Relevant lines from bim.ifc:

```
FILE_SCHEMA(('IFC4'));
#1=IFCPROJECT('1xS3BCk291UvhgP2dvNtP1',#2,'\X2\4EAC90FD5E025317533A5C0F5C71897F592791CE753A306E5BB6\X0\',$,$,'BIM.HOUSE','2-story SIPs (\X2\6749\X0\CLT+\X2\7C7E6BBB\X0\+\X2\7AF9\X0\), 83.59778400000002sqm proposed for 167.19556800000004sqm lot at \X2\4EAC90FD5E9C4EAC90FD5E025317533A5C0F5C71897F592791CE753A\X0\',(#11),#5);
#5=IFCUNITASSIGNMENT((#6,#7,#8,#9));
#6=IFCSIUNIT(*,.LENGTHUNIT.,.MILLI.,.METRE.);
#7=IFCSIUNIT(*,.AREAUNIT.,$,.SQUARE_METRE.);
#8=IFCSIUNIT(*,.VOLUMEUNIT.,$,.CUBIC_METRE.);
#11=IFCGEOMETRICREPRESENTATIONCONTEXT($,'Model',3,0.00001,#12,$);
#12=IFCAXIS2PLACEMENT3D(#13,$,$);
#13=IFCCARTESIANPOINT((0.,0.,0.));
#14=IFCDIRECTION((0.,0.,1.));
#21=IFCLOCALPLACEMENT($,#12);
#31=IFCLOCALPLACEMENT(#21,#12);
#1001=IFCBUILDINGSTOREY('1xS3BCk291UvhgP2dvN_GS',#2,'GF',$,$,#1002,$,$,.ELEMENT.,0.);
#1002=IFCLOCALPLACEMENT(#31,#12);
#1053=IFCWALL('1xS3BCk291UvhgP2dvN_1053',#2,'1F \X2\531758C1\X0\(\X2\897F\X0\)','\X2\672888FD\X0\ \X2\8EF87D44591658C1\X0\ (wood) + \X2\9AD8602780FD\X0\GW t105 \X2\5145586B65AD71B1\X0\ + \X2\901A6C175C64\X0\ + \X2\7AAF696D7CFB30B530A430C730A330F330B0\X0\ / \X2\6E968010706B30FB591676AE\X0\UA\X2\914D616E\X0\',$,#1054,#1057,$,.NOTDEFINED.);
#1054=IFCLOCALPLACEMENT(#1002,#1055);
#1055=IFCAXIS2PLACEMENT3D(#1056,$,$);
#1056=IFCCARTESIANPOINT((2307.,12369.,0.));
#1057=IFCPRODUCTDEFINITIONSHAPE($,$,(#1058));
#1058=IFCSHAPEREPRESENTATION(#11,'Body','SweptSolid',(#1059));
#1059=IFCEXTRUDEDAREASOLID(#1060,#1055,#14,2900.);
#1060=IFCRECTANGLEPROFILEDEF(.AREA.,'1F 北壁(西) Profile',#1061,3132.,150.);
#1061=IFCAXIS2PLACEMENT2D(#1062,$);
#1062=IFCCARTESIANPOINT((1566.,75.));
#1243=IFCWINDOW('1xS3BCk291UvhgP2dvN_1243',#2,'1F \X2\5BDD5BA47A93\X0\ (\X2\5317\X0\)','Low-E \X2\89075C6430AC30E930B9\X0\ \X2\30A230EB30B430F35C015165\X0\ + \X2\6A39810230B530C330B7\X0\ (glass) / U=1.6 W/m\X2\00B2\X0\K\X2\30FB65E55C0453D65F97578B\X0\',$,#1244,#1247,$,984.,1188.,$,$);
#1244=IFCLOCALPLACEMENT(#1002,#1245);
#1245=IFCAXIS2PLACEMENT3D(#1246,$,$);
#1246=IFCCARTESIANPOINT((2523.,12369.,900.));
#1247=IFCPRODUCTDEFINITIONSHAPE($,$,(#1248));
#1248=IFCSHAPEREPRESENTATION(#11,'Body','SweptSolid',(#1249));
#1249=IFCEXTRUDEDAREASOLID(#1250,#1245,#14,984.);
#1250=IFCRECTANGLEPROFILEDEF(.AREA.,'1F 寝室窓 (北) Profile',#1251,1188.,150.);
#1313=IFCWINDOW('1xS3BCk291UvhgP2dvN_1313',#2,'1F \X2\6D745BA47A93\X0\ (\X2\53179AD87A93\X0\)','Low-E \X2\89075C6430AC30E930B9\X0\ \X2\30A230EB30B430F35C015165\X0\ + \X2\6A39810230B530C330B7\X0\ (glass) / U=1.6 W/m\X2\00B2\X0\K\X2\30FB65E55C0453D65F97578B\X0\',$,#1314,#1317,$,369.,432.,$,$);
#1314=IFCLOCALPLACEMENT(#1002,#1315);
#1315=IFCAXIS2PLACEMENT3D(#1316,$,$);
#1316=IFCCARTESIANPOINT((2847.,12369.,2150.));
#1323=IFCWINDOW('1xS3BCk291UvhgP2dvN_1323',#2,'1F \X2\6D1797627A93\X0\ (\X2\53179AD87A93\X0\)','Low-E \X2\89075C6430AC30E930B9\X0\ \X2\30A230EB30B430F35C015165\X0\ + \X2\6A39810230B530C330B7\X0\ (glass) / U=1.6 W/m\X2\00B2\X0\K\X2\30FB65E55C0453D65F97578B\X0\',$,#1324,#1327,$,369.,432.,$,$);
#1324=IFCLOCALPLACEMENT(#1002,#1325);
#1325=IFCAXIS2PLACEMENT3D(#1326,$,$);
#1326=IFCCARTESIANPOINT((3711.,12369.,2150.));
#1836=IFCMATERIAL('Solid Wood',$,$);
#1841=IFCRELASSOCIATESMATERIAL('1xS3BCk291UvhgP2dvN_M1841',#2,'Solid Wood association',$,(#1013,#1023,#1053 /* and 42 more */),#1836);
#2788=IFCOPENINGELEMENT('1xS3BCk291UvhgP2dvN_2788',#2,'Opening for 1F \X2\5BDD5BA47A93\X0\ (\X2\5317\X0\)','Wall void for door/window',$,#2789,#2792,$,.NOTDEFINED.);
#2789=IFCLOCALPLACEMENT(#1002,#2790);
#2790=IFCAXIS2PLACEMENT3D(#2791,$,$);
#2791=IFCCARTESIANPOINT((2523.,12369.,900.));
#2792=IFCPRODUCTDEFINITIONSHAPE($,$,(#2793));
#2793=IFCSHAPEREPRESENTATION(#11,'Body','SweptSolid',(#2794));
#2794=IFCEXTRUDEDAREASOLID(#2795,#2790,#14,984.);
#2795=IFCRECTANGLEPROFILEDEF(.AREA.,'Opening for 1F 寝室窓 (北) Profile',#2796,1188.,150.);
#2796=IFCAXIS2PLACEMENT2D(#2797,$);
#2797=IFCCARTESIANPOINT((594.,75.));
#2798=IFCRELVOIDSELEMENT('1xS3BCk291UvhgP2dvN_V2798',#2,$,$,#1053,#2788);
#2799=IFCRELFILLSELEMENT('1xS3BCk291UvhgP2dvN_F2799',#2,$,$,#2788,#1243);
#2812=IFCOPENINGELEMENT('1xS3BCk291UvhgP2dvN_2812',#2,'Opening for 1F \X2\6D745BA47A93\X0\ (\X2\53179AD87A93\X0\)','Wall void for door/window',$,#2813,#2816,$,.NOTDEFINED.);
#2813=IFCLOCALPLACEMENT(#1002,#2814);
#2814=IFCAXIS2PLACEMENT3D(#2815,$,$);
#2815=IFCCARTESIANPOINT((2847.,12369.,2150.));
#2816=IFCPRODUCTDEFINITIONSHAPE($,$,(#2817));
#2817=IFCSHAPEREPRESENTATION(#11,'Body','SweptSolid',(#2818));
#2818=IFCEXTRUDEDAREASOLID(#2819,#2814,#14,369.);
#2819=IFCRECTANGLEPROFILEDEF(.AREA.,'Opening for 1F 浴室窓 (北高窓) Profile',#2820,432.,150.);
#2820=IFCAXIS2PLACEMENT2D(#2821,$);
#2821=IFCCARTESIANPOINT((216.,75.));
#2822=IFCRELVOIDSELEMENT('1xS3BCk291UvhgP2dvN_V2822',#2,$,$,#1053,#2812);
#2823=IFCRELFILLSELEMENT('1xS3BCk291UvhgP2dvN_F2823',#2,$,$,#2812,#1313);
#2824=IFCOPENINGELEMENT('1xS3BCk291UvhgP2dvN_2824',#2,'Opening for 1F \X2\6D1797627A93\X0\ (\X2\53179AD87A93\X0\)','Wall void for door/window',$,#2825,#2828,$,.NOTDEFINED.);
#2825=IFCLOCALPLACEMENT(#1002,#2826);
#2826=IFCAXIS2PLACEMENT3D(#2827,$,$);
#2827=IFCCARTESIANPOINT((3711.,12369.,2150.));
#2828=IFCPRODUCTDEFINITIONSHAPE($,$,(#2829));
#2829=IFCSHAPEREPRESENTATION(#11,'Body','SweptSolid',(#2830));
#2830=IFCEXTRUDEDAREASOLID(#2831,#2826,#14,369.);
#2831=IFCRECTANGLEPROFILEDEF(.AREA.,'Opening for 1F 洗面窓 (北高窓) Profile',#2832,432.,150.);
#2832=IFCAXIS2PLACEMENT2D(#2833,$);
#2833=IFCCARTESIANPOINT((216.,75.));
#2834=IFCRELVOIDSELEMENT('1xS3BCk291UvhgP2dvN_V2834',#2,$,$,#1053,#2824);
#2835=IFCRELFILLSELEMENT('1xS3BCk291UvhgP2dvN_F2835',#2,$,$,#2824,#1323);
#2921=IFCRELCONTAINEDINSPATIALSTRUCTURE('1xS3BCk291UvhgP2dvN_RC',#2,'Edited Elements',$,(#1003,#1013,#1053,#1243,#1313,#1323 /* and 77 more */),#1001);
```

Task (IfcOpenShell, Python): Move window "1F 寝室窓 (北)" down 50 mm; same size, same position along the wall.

```python
import numpy as np
import ifcopenshell
import ifcopenshell.api.geometry
import ifcopenshell.util.placement
import ifcopenshell.util.unit

model = ifcopenshell.open("bim.ifc")
unit_scale = ifcopenshell.util.unit.calculate_unit_scale(model)

window = model.by_guid("1xS3BCk291UvhgP2dvN_1243")
opening = window.FillsVoids[0].RelatingOpeningElement
dz = -0.05 / unit_scale

shift = np.array([0.0, 0.0, dz])
# The window is not placed relative to its opening, so move both.
for product in (opening, window):
    matrix = ifcopenshell.util.placement.get_local_placement(product.ObjectPlacement)
    matrix[:3, 3] += shift
    ifcopenshell.api.geometry.edit_object_placement(model, product=product, matrix=matrix, is_si=False)

print(f"moved by {dz * unit_scale:+.3f} m")

model.write("bim_v2.ifc")
```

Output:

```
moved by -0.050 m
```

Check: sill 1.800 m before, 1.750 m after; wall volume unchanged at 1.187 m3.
